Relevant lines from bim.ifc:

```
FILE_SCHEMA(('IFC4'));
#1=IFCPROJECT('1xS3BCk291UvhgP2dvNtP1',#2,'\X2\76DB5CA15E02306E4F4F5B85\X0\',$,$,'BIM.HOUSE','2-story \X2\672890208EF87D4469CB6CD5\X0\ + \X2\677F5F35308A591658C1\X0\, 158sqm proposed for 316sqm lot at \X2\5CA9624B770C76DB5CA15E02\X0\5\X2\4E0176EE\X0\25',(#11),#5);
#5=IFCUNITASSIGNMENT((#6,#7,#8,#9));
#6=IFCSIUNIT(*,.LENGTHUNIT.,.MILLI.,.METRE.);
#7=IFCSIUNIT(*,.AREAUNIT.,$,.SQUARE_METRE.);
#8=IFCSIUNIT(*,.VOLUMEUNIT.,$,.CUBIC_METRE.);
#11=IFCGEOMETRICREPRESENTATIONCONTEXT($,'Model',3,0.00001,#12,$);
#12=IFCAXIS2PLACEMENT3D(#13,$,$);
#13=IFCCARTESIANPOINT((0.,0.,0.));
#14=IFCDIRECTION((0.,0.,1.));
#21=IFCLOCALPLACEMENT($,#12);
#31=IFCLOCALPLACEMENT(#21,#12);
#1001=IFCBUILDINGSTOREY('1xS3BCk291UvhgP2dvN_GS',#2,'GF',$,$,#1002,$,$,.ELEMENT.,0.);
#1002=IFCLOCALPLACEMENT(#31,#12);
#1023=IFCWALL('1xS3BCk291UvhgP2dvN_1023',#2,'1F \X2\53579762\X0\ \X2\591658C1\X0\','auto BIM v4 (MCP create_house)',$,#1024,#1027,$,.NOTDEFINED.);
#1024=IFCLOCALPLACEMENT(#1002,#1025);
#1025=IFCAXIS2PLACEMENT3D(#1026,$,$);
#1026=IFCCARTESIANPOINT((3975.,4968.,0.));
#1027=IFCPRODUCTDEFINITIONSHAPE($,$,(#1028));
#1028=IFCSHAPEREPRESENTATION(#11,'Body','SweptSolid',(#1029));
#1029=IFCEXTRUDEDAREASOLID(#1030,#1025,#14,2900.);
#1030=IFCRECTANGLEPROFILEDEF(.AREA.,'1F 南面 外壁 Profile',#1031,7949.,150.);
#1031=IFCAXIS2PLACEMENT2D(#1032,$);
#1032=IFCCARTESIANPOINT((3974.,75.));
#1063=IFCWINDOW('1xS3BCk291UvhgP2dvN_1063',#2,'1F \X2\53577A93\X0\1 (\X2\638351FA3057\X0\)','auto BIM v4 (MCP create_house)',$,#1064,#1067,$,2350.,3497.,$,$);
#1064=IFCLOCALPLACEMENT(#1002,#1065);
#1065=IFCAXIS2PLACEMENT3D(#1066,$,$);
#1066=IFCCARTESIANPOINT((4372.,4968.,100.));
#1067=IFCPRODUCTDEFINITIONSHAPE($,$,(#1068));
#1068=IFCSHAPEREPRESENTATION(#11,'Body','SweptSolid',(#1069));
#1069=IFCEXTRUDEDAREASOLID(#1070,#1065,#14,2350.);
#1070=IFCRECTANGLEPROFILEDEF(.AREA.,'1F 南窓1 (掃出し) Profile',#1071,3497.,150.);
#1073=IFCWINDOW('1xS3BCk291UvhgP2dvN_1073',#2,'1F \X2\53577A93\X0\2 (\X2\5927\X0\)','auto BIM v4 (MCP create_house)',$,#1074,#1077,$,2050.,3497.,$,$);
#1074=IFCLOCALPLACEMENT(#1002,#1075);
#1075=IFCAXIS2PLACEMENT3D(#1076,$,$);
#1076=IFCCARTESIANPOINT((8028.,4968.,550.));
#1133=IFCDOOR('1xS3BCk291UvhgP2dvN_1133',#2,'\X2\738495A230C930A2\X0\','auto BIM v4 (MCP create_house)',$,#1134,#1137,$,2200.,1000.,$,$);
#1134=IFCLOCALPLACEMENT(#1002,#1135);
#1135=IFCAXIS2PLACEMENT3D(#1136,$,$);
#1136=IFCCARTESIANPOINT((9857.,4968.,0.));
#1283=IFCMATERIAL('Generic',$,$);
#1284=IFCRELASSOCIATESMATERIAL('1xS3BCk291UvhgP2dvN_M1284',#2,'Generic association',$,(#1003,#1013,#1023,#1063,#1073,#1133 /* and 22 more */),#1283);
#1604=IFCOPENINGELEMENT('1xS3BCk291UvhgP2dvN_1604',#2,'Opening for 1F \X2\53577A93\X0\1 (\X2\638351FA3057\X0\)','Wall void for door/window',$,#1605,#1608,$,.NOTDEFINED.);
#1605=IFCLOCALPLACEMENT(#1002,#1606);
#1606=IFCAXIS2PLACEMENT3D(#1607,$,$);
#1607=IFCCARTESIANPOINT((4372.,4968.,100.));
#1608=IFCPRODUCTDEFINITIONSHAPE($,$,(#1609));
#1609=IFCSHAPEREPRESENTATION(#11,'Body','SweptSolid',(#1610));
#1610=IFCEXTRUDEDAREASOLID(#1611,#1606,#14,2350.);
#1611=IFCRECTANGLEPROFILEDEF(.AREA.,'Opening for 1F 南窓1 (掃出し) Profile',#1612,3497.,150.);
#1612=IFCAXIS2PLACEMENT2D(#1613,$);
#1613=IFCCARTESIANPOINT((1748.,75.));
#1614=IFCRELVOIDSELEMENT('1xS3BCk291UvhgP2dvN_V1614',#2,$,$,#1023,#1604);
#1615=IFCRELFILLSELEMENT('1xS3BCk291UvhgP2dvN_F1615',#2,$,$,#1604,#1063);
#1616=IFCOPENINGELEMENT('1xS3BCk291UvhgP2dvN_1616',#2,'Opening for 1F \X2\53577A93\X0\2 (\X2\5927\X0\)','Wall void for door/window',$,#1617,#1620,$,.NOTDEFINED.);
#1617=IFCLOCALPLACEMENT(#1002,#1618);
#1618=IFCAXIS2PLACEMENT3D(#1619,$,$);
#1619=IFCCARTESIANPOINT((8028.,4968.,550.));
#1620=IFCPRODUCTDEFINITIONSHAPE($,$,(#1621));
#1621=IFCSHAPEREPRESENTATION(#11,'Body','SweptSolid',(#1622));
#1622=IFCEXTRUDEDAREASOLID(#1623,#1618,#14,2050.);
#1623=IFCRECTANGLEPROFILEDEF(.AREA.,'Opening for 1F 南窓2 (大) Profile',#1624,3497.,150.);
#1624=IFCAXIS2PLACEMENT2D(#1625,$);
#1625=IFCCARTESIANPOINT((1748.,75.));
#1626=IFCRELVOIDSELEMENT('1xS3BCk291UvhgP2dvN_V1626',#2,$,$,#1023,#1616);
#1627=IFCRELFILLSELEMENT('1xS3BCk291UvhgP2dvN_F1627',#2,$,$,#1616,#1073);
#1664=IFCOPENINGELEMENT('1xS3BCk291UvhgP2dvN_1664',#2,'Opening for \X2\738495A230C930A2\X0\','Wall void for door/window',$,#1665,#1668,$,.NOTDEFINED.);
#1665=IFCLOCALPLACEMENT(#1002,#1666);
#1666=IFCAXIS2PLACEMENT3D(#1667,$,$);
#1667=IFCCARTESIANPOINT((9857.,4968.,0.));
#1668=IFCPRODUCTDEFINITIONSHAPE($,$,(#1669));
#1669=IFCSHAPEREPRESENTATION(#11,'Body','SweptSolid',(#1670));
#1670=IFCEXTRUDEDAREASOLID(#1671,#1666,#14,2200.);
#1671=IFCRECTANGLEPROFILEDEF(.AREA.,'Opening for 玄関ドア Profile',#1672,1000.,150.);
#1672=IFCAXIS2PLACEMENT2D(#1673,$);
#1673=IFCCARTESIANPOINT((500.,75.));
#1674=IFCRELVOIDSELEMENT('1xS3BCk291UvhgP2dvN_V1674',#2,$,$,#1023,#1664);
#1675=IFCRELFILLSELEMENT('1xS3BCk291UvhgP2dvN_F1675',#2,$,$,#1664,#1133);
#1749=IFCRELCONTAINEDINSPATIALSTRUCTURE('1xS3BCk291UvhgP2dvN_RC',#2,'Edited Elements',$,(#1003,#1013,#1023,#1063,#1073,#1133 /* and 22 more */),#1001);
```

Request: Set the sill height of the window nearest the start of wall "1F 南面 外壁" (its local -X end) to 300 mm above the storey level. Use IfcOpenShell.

```python
import numpy as np
import ifcopenshell
import ifcopenshell.api.geometry
import ifcopenshell.geom
import ifcopenshell.util.element
import ifcopenshell.util.placement
import ifcopenshell.util.shape
import ifcopenshell.util.unit

model = ifcopenshell.open("bim.ifc")
unit_scale = ifcopenshell.util.unit.calculate_unit_scale(model)

window = model.by_id(1063)
opening = window.FillsVoids[0].RelatingOpeningElement
storey = ifcopenshell.util.element.get_container(window, ifc_class="IfcBuildingStorey")
level = ifcopenshell.util.placement.get_local_placement(storey.ObjectPlacement)[2, 3]

# The opening's origin need not be at the sill, so measure its lowest point.
shape = ifcopenshell.geom.create_shape(ifcopenshell.geom.settings(), opening)
bottom = ifcopenshell.util.shape.get_shape_bottom_elevation(shape, shape.geometry) / unit_scale
dz = level + 0.3 / unit_scale - bottom

shift = np.array([0.0, 0.0, dz])
# The window is not placed relative to its opening, so move both.
for product in (opening, window):
    matrix = ifcopenshell.util.placement.get_local_placement(product.ObjectPlacement)
    matrix[:3, 3] += shift
    ifcopenshell.api.geometry.edit_object_placement(model, product=product, matrix=matrix, is_si=False)

print(f"moved by {dz * unit_scale:+.3f} m")

model.write("bim_edited.ifc")
```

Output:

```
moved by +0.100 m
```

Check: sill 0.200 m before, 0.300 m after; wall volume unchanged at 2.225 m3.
